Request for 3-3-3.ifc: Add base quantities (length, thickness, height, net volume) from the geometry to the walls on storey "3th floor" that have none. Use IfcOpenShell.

First a look at what the model holds.

```python
import ifcopenshell
import ifcopenshell.util.element
import ifcopenshell.util.unit

model = ifcopenshell.open("3-3-3.ifc")
print(model.schema)
for unit_type in ("LENGTHUNIT", "AREAUNIT", "VOLUMEUNIT"):
    print(unit_type, ifcopenshell.util.unit.calculate_unit_scale(model, unit_type))
storey = next(s for s in model.by_type("IfcBuildingStorey") if s.Name == "3th floor")
walls = [e for e in ifcopenshell.util.element.get_decomposition(storey) if e.is_a("IfcWall")]
for e in sorted(walls, key=lambda e: e.id()):
    print(e.id(), e.is_a(), e.Name, list(ifcopenshell.util.element.get_psets(e, qtos_only=True)), sep=" | ")
```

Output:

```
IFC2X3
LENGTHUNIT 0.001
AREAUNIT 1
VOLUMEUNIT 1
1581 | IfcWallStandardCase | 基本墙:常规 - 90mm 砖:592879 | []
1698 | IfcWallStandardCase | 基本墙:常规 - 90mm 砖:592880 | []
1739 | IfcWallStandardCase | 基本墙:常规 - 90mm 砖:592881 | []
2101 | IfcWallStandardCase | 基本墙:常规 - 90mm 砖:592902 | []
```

```python
import ifcopenshell
import ifcopenshell.api.pset
import ifcopenshell.geom
import ifcopenshell.util.element
import ifcopenshell.util.shape
import ifcopenshell.util.unit

model = ifcopenshell.open("3-3-3.ifc")
unit_scale = ifcopenshell.util.unit.calculate_unit_scale(model)
volume_scale = ifcopenshell.util.unit.calculate_unit_scale(model, "VOLUMEUNIT")
settings = ifcopenshell.geom.settings()

storey = next(s for s in model.by_type("IfcBuildingStorey") if s.Name == "3th floor")
walls = [e for e in ifcopenshell.util.element.get_decomposition(storey) if e.is_a("IfcWall")]

for e in sorted(walls, key=lambda e: e.id()):
    if ifcopenshell.util.element.get_psets(e, qtos_only=True, should_inherit=False):
        continue
    # Geometry comes back in metres, in the element's own axes.
    shape = ifcopenshell.geom.create_shape(settings, e)
    values = {
        "Length": ifcopenshell.util.shape.get_x(shape.geometry) / unit_scale,
        "Width": ifcopenshell.util.shape.get_y(shape.geometry) / unit_scale,
        "Height": ifcopenshell.util.shape.get_z(shape.geometry) / unit_scale,
        "NetVolume": ifcopenshell.util.shape.get_volume(shape.geometry) / volume_scale,
    }
    qto = ifcopenshell.api.pset.add_qto(model, product=e, name="BaseQuantities")
    ifcopenshell.api.pset.edit_qto(model, qto=qto, properties=values)
    print(e.id(), {k: round(v, 3) for k, v in values.items()})

model.write("3-3-3_v2.ifc")
```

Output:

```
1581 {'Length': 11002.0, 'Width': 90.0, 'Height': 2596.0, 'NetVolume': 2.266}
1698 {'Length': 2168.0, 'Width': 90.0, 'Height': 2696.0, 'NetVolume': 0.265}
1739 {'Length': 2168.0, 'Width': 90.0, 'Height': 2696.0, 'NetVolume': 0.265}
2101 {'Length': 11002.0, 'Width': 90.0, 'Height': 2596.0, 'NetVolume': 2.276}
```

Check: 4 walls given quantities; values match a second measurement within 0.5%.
